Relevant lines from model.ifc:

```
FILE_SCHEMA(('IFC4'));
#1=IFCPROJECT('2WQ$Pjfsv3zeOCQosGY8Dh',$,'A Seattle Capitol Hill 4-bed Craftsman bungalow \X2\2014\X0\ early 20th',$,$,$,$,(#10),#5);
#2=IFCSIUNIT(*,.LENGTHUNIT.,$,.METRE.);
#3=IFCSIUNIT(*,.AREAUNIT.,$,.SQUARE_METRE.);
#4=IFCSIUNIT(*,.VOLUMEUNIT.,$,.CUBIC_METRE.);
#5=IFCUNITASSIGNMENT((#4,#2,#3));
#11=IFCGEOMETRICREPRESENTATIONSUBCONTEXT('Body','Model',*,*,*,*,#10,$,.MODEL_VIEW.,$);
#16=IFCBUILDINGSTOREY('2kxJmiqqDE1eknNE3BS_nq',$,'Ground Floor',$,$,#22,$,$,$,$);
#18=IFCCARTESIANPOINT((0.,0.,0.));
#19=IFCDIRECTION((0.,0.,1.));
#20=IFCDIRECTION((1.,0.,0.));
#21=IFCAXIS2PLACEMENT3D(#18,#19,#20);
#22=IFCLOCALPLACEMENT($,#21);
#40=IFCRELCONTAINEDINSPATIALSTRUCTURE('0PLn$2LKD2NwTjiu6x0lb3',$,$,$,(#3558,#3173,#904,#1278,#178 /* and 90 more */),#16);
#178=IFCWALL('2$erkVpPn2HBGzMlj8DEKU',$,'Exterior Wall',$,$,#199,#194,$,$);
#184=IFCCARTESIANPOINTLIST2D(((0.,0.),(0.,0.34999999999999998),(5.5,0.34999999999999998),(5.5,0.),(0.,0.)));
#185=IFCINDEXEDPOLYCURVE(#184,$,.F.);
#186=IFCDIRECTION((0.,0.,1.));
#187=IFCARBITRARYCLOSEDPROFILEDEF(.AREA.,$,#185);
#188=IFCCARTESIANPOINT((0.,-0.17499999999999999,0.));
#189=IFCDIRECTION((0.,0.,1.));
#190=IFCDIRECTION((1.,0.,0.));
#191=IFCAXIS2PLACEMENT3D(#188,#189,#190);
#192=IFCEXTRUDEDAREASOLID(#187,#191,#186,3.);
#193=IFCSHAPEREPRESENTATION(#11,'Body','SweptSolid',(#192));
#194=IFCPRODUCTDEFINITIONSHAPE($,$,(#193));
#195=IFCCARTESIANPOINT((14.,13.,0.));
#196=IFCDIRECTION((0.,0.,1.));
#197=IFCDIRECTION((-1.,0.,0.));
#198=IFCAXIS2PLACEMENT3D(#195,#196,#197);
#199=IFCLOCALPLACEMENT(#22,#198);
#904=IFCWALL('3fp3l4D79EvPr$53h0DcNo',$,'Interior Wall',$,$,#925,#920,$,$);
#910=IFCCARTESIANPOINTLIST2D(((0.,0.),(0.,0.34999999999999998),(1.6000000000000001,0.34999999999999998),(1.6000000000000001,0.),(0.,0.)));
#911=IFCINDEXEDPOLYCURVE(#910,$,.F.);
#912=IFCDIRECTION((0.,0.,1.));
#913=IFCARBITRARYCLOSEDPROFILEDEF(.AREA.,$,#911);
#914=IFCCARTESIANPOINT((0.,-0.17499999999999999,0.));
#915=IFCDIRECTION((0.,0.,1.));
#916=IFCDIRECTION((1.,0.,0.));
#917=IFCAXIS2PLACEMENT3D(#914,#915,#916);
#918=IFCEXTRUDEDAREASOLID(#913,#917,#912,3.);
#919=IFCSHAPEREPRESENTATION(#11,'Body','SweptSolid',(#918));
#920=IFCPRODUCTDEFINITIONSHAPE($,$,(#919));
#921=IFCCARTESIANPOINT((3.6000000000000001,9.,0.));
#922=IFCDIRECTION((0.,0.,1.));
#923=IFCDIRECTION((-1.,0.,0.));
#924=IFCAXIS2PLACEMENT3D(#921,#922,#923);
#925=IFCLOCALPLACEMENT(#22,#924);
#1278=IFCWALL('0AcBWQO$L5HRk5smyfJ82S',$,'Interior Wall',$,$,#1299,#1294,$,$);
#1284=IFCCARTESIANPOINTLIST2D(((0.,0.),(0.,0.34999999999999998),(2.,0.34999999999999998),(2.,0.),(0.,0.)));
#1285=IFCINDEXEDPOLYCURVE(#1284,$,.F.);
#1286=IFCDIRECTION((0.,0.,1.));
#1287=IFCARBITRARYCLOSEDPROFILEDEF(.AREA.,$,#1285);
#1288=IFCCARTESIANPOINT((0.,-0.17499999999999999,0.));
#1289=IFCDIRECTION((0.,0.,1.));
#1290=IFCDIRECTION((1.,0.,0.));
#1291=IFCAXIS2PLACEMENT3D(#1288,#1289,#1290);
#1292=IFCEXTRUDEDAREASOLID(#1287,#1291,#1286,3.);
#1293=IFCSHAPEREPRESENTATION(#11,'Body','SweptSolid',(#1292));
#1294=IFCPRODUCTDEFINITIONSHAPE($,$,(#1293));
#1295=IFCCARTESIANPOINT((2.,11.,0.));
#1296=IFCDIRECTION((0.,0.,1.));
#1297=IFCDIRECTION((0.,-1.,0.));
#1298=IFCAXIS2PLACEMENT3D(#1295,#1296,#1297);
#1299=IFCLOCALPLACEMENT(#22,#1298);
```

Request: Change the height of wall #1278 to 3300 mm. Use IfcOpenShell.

```python
import ifcopenshell
import ifcopenshell.geom
import ifcopenshell.util.representation
import ifcopenshell.util.shape

model = ifcopenshell.open("model.ifc")
settings = ifcopenshell.geom.settings()


def volume(element):
    """Net volume in cubic metres, openings subtracted."""
    shape = ifcopenshell.geom.create_shape(settings, element)
    return ifcopenshell.util.shape.get_volume(shape.geometry)


wall = model.by_id(1278)
before = volume(wall)

body = ifcopenshell.util.representation.get_representation(wall, "Model", "Body")
solid = body.Items[0]
old_height = solid.Depth
solid.Depth = 3.3
after = volume(wall)

print(f"height {old_height:g} -> {solid.Depth:g}, volume {before:.3f} -> {after:.3f} m3")

model.write("model_updated.ifc")
```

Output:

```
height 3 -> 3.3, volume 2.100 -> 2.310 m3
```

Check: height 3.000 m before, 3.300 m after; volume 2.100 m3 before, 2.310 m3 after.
